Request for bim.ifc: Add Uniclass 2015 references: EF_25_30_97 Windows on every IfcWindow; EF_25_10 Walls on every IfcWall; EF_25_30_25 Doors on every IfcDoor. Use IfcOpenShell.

First a look at what the model holds.

```python
import ifcopenshell

model = ifcopenshell.open("bim.ifc")
print(model.schema)
print("classifications:", [c.Name for c in model.by_type("IfcClassification")])
for ifc_class in ("IfcDoor", "IfcRoof", "IfcStair", "IfcWall", "IfcWindow"):
    print(ifc_class, len(model.by_type(ifc_class)))
```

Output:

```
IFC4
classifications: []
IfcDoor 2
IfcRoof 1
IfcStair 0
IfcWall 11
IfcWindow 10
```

```python
import ifcopenshell
import ifcopenshell.api.classification

model = ifcopenshell.open("bim.ifc")

system = ifcopenshell.api.classification.add_classification(model, classification="Uniclass 2015")

codes = {
    "IfcWindow": ("EF_25_30_97", "Windows"),
    "IfcWall": ("EF_25_10", "Walls"),
    "IfcDoor": ("EF_25_30_25", "Doors"),
}
for ifc_class, (code, name) in codes.items():
    products = model.by_type(ifc_class)
    ifcopenshell.api.classification.add_reference(
        model, products=products, classification=system, identification=code, name=name
    )
    print(code, len(products))

model.write("bim_v2.ifc")
```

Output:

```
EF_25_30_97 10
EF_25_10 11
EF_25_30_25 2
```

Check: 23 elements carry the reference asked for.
